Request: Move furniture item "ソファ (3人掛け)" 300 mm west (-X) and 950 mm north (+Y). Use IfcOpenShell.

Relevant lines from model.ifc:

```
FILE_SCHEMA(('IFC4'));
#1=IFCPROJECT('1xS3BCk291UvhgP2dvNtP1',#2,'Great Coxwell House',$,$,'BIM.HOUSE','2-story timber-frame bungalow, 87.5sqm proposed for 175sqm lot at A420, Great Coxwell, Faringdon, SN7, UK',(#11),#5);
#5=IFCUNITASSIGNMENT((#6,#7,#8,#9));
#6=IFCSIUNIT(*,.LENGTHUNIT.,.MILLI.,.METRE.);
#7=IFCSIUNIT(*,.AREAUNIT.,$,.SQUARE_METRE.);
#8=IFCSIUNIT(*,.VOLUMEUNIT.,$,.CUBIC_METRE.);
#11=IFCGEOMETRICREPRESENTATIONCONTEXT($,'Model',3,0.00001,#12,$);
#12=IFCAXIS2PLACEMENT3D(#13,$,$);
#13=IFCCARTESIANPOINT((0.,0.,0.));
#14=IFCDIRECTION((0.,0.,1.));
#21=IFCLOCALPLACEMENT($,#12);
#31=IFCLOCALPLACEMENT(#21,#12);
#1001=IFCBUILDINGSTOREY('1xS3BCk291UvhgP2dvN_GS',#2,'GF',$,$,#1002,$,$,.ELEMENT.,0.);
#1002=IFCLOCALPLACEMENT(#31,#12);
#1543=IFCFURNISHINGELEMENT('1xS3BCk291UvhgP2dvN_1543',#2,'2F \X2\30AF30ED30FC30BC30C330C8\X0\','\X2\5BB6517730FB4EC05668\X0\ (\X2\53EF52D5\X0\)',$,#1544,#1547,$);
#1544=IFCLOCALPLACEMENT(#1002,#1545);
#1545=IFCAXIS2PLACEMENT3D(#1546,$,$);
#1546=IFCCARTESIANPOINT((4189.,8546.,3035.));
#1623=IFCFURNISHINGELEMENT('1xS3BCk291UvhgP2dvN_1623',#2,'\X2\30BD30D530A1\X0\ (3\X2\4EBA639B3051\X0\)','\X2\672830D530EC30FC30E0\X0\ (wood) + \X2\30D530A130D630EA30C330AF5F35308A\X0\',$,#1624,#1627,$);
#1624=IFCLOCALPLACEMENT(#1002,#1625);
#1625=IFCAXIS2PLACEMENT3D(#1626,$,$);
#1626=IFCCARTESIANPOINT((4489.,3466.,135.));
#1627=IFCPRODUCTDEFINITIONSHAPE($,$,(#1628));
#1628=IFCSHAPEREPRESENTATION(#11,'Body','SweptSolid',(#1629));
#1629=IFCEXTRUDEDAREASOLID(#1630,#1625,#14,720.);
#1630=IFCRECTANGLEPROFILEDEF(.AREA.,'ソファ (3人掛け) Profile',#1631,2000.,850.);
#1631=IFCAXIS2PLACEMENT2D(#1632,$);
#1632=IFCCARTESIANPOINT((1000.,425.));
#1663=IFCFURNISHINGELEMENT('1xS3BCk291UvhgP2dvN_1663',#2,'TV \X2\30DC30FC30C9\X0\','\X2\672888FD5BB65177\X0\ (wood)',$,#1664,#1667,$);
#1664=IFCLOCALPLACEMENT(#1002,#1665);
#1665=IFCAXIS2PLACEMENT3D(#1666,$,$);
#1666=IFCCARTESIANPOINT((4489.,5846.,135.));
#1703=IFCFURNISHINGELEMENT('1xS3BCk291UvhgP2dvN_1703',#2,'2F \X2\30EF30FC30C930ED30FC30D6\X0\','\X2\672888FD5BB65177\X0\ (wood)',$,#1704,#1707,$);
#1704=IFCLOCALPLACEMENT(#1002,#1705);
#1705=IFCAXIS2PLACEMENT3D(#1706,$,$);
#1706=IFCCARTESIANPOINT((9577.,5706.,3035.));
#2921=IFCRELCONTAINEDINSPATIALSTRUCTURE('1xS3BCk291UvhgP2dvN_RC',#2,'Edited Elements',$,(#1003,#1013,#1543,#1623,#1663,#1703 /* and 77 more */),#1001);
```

```python
import ifcopenshell
import ifcopenshell.api.geometry
import ifcopenshell.util.placement

model = ifcopenshell.open("model.ifc")

item = model.by_id(1623)
matrix = ifcopenshell.util.placement.get_local_placement(item.ObjectPlacement)
matrix[0, 3] -= 300.0
matrix[1, 3] += 950.0
ifcopenshell.api.geometry.edit_object_placement(model, product=item, matrix=matrix, is_si=False)

print(ifcopenshell.util.placement.get_local_placement(item.ObjectPlacement).round(3) + 0.0)

model.write("model-out.ifc")
```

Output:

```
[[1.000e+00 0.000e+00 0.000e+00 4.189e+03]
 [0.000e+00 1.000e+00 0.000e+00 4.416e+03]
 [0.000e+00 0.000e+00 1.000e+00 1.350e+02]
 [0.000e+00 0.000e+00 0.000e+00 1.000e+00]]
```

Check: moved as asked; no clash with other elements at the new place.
